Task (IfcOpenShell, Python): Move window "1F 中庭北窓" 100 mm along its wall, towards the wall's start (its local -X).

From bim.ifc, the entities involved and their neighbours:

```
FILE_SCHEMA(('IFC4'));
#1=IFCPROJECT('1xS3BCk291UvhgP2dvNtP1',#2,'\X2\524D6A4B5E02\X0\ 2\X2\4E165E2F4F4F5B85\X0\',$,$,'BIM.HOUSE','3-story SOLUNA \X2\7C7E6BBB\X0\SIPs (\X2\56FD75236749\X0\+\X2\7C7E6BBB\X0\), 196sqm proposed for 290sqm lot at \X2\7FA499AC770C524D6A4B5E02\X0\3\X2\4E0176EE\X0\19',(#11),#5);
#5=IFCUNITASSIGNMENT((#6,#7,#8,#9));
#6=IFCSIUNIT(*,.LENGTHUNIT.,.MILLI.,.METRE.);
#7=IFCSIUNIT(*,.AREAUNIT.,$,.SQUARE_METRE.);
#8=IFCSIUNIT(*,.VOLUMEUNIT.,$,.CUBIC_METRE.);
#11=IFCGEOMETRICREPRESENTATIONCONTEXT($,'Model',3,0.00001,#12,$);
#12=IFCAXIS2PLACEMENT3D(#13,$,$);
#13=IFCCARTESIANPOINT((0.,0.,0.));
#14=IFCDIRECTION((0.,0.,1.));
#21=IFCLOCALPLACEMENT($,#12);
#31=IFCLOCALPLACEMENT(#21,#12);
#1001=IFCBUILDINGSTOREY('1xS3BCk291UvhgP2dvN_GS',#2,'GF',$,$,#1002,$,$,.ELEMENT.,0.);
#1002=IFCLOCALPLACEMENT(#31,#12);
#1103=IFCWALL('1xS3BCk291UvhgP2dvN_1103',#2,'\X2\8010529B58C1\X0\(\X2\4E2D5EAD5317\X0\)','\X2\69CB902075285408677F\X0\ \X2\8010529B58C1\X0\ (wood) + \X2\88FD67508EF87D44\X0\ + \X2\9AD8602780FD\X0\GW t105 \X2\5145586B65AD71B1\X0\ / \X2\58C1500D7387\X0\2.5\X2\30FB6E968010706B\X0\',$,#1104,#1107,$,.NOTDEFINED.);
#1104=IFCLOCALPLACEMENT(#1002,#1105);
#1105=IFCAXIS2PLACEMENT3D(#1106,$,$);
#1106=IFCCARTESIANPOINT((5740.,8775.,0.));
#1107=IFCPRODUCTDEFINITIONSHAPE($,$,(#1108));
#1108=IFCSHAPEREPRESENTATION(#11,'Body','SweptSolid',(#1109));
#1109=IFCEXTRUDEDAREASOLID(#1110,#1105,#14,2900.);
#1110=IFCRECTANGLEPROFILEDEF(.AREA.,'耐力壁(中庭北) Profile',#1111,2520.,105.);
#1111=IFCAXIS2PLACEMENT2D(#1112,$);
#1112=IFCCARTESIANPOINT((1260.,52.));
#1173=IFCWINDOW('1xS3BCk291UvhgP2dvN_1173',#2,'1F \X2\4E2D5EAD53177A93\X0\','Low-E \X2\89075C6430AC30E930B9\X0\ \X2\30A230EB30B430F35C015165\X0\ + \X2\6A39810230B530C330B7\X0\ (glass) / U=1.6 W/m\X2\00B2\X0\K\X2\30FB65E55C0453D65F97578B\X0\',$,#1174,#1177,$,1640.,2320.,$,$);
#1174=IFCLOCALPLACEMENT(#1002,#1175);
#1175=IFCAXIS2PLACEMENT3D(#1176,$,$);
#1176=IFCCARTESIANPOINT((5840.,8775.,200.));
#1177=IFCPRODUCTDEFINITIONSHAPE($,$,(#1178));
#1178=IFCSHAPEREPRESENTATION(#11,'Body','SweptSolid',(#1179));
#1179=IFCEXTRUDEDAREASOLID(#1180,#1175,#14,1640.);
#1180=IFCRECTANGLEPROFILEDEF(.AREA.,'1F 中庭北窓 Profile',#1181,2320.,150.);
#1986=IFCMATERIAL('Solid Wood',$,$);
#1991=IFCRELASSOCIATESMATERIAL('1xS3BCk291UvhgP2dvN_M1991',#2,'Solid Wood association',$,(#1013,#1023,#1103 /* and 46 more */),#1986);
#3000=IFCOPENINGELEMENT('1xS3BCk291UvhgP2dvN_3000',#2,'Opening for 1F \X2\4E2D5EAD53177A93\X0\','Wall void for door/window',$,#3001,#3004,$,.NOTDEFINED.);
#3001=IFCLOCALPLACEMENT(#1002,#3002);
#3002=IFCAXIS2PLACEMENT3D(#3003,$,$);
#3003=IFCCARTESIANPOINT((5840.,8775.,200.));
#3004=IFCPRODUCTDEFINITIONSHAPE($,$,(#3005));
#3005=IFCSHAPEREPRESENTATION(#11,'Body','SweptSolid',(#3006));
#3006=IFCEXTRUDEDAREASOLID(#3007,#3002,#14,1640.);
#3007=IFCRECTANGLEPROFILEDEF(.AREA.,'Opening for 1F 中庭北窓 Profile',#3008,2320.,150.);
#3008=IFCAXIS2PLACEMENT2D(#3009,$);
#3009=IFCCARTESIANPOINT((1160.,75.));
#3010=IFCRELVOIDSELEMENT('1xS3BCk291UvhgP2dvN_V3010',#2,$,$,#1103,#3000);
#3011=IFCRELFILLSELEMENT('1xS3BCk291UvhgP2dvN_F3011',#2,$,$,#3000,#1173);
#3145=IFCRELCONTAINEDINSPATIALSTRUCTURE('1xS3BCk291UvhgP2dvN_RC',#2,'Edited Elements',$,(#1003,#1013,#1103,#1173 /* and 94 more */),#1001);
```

```python
import ifcopenshell
import ifcopenshell.api.geometry
import ifcopenshell.util.placement
import ifcopenshell.util.unit

model = ifcopenshell.open("bim.ifc")
unit_scale = ifcopenshell.util.unit.calculate_unit_scale(model)

window = model.by_guid("1xS3BCk291UvhgP2dvN_1173")
opening = window.FillsVoids[0].RelatingOpeningElement
wall = opening.VoidsElements[0].RelatingBuildingElement

wall_matrix = ifcopenshell.util.placement.get_local_placement(wall.ObjectPlacement)
shift = wall_matrix[:3, 0] * -0.1 / unit_scale
before = ifcopenshell.util.placement.get_local_placement(window.ObjectPlacement)[:3, 3].copy()

# The window is not placed relative to its opening, so move both.
for product in (opening, window):
    matrix = ifcopenshell.util.placement.get_local_placement(product.ObjectPlacement)
    matrix[:3, 3] += shift
    ifcopenshell.api.geometry.edit_object_placement(model, product=product, matrix=matrix, is_si=False)

after = ifcopenshell.util.placement.get_local_placement(window.ObjectPlacement)[:3, 3]
print("window moved by", (after - before).round(3) + 0.0)

model.write("bim_v2.ifc")
```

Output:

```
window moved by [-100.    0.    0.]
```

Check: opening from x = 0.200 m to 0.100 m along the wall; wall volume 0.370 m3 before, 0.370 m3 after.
